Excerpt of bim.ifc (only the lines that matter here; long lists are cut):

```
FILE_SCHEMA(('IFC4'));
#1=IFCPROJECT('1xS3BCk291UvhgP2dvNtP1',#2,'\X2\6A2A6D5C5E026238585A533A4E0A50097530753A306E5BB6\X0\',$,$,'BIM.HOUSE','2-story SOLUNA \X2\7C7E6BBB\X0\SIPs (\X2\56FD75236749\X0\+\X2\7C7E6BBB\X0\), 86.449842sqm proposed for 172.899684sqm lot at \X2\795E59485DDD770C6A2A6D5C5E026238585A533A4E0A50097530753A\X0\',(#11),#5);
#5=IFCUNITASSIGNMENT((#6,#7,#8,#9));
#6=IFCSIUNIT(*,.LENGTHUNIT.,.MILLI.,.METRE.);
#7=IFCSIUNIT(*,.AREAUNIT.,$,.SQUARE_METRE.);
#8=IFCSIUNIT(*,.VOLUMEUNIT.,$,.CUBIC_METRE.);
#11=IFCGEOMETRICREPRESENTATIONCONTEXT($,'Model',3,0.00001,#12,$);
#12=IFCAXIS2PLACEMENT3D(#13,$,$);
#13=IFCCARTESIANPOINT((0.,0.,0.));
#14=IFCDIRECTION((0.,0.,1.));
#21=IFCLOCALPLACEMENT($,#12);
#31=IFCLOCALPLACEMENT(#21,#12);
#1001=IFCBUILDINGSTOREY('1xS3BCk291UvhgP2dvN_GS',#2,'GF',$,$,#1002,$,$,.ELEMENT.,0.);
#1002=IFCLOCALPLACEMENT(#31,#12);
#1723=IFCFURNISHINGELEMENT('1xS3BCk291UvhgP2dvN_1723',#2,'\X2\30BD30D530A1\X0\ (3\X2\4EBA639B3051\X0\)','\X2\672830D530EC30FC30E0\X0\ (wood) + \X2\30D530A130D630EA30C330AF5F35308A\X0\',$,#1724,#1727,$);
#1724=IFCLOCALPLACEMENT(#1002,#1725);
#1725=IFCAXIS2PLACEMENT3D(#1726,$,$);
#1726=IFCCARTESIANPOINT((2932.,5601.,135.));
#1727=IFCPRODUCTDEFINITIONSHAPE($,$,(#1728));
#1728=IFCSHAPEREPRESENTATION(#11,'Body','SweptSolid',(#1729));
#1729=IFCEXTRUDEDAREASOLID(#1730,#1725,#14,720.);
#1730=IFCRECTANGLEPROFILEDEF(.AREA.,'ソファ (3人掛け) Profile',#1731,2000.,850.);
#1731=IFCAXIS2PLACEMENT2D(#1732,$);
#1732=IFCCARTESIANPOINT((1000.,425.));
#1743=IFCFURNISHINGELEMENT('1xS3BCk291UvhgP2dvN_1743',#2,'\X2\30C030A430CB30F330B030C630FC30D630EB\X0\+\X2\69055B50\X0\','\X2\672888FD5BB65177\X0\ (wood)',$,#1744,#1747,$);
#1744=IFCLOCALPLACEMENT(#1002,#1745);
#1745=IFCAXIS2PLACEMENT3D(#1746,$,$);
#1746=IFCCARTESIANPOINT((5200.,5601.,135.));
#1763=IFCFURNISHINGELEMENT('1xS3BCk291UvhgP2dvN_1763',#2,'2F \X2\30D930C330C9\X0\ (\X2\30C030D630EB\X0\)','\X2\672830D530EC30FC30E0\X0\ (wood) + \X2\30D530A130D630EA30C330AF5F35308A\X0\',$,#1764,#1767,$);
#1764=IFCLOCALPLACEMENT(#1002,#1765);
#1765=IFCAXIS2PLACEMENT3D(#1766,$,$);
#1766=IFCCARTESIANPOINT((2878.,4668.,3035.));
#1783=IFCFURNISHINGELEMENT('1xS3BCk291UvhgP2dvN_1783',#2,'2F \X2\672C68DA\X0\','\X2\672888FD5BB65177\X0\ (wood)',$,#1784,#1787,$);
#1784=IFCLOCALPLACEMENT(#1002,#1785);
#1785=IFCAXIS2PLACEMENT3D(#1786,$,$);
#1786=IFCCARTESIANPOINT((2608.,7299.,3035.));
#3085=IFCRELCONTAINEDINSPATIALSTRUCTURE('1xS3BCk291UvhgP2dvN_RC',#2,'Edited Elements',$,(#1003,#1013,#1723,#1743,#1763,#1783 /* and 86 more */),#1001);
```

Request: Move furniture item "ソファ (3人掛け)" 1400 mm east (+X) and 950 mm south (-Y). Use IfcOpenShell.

```python
import ifcopenshell
import ifcopenshell.api.geometry
import ifcopenshell.util.placement

model = ifcopenshell.open("bim.ifc")

item = model.by_guid("1xS3BCk291UvhgP2dvN_1723")
matrix = ifcopenshell.util.placement.get_local_placement(item.ObjectPlacement)
matrix[0, 3] += 1400.0
matrix[1, 3] -= 950.0
ifcopenshell.api.geometry.edit_object_placement(model, product=item, matrix=matrix, is_si=False)

print(ifcopenshell.util.placement.get_local_placement(item.ObjectPlacement).round(3) + 0.0)

model.write("bim_v2.ifc")
```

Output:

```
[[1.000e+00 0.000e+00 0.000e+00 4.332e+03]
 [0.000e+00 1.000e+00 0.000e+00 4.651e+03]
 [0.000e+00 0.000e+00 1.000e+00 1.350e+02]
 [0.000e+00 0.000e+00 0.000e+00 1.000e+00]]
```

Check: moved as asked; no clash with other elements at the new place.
